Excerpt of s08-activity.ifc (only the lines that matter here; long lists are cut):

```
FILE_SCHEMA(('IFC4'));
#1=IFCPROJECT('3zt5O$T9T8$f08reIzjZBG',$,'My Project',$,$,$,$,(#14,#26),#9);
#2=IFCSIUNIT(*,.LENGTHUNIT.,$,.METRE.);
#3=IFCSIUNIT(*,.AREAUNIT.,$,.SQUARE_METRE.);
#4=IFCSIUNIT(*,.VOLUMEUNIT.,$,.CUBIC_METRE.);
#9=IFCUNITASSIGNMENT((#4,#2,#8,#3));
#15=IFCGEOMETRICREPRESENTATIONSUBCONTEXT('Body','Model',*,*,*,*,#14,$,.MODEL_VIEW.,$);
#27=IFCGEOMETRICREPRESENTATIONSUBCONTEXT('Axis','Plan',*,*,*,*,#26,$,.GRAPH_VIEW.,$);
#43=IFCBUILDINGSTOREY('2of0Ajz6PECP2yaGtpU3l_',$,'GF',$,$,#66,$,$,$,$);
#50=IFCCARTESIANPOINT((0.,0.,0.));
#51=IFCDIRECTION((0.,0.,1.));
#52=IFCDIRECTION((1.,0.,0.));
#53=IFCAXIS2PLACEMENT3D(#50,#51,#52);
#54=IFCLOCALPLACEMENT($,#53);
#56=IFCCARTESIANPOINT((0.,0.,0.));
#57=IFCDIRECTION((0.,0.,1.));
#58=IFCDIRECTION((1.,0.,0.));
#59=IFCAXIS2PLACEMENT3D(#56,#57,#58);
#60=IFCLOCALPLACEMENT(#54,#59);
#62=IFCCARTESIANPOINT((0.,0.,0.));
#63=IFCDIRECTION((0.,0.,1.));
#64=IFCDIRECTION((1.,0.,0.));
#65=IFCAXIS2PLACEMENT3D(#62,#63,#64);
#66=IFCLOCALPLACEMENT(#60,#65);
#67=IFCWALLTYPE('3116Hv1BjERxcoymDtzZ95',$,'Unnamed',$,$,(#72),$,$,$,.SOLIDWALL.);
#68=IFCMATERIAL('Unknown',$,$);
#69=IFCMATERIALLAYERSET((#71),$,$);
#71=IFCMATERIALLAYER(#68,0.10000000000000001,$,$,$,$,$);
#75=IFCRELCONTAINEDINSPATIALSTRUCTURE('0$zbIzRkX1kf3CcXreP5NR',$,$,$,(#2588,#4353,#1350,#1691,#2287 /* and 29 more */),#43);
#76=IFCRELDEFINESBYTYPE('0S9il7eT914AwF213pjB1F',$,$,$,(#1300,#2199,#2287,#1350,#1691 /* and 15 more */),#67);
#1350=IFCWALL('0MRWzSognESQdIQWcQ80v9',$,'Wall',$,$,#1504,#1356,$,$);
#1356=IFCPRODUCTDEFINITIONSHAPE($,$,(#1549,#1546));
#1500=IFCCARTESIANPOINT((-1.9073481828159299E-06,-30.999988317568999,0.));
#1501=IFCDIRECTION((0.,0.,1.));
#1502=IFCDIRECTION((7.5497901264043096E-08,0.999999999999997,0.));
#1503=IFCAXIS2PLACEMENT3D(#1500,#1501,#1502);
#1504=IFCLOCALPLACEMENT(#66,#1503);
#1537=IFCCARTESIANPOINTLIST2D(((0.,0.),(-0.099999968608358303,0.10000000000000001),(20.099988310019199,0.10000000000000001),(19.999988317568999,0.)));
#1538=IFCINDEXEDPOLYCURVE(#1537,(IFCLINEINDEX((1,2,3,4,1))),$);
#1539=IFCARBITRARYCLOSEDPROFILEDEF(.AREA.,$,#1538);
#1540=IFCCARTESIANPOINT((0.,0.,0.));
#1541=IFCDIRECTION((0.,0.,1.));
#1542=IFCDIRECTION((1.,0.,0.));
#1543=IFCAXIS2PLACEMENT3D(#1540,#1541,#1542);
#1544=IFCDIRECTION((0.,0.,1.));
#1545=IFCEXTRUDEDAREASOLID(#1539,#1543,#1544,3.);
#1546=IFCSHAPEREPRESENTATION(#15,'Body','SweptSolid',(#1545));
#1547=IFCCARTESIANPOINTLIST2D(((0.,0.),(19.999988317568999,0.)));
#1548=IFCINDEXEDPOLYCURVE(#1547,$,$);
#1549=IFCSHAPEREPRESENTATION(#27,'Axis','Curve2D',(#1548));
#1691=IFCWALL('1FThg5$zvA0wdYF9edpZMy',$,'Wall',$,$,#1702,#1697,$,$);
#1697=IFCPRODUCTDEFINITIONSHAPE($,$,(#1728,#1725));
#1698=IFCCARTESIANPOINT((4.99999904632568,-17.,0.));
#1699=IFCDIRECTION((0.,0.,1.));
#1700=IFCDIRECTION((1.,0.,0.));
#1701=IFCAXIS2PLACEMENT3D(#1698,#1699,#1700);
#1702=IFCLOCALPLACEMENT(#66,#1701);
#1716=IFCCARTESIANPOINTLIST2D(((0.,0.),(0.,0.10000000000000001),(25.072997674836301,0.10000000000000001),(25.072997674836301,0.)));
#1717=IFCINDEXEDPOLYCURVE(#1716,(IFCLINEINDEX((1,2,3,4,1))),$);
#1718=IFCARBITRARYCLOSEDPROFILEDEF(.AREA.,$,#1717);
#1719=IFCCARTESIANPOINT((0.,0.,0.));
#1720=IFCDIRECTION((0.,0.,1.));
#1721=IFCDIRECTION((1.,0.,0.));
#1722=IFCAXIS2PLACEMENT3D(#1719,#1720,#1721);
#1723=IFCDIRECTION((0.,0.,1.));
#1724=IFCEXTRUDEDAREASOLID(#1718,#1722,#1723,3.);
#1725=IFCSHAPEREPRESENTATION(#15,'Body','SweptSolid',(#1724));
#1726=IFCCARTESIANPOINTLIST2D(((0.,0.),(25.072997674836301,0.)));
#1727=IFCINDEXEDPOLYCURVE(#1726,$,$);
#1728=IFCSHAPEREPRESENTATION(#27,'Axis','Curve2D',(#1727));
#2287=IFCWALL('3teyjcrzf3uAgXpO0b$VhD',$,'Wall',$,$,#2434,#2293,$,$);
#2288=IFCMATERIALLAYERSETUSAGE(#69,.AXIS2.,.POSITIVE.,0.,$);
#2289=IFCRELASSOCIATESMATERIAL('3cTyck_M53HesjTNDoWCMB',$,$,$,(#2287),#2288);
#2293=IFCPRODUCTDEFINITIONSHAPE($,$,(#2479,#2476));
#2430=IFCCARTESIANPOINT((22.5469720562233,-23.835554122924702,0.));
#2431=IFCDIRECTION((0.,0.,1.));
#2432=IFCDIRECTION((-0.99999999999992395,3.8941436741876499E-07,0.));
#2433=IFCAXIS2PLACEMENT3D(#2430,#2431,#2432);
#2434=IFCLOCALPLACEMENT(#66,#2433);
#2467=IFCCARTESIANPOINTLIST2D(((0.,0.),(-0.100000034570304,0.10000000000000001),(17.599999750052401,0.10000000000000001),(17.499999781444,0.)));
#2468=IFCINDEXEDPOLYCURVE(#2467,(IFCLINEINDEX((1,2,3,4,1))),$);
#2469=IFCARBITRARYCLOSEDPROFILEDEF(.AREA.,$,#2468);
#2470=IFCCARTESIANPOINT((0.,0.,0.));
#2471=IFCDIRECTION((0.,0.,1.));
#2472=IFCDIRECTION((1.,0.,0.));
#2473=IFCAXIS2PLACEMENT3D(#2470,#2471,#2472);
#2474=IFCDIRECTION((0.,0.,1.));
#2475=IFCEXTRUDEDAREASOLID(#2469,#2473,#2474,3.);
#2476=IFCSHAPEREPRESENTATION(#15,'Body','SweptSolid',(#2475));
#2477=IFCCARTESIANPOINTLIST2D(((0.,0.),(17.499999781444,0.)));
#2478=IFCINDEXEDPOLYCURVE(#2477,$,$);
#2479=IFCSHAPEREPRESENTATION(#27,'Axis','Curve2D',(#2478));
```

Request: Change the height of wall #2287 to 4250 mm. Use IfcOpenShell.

```python
import ifcopenshell
import ifcopenshell.geom
import ifcopenshell.util.representation
import ifcopenshell.util.shape

model = ifcopenshell.open("s08-activity.ifc")
settings = ifcopenshell.geom.settings()


def volume(element):
    """Net volume in cubic metres, openings subtracted."""
    shape = ifcopenshell.geom.create_shape(settings, element)
    return ifcopenshell.util.shape.get_volume(shape.geometry)


wall = model.by_id(2287)
before = volume(wall)

body = ifcopenshell.util.representation.get_representation(wall, "Model", "Body")
solid = body.Items[0]
old_height = solid.Depth
solid.Depth = 4.25
after = volume(wall)

print(f"height {old_height:g} -> {solid.Depth:g}, volume {before:.3f} -> {after:.3f} m3")

model.write("s08-activity_v2.ifc")
```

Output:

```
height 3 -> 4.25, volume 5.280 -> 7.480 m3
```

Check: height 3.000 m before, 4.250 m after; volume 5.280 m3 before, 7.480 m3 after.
